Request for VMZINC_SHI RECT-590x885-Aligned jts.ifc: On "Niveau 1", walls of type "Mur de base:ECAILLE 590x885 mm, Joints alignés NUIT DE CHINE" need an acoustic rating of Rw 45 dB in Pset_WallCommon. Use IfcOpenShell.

First a look at what the model holds.

```python
import ifcopenshell
import ifcopenshell.util.element

model = ifcopenshell.open("VMZINC_SHI RECT-590x885-Aligned jts.ifc")
print(model.schema)
storey = next(s for s in model.by_type("IfcBuildingStorey") if s.Name == "Niveau 1")
walls = [e for e in ifcopenshell.util.element.get_decomposition(storey) if e.is_a("IfcWall")]
seen = {}
for e in walls:
    element_type = ifcopenshell.util.element.get_type(e)
    key = (element_type.Name if element_type != e and element_type else None, ifcopenshell.util.element.get_pset(e, "Pset_WallCommon", "AcousticRating"))
    seen[key] = seen.get(key, 0) + 1
for (name, value), count in sorted(seen.items(), key=str):
    print(count, "x", name, "|", value)
```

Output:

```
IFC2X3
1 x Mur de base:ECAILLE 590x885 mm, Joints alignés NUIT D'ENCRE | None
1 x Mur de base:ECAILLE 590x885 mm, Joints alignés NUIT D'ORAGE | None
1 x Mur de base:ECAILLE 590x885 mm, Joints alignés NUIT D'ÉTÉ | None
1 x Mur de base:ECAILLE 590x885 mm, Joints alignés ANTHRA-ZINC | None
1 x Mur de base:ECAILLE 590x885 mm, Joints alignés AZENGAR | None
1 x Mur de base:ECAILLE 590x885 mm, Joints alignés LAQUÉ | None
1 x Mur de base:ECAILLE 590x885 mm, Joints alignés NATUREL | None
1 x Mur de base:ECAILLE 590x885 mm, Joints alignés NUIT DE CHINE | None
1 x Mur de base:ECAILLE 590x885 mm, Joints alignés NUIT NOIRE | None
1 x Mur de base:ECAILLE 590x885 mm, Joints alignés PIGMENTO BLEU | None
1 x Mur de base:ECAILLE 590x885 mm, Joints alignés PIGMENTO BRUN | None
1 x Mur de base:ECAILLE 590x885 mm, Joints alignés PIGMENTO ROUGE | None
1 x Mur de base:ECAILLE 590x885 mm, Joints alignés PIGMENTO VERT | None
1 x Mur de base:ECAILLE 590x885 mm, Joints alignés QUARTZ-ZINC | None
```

```python
import ifcopenshell
import ifcopenshell.api.pset
import ifcopenshell.util.element

model = ifcopenshell.open("VMZINC_SHI RECT-590x885-Aligned jts.ifc")

storey = next(s for s in model.by_type("IfcBuildingStorey") if s.Name == "Niveau 1")
walls = [e for e in ifcopenshell.util.element.get_decomposition(storey) if e.is_a("IfcWall")]

count = 0
for e in walls:
    element_type = ifcopenshell.util.element.get_type(e)
    if element_type in (None, e) or element_type.Name != "Mur de base:ECAILLE 590x885 mm, Joints alignés NUIT DE CHINE":
        continue
    # add_pset returns the element's existing set when there is one.
    pset = ifcopenshell.api.pset.add_pset(model, product=e, name="Pset_WallCommon")
    ifcopenshell.api.pset.edit_pset(model, pset=pset, properties={"AcousticRating": "Rw 45 dB"})
    count += 1

print(count, "walls updated")

model.write("VMZINC_SHI RECT-590x885-Aligned jts_edited.ifc")
```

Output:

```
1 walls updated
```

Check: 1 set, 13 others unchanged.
